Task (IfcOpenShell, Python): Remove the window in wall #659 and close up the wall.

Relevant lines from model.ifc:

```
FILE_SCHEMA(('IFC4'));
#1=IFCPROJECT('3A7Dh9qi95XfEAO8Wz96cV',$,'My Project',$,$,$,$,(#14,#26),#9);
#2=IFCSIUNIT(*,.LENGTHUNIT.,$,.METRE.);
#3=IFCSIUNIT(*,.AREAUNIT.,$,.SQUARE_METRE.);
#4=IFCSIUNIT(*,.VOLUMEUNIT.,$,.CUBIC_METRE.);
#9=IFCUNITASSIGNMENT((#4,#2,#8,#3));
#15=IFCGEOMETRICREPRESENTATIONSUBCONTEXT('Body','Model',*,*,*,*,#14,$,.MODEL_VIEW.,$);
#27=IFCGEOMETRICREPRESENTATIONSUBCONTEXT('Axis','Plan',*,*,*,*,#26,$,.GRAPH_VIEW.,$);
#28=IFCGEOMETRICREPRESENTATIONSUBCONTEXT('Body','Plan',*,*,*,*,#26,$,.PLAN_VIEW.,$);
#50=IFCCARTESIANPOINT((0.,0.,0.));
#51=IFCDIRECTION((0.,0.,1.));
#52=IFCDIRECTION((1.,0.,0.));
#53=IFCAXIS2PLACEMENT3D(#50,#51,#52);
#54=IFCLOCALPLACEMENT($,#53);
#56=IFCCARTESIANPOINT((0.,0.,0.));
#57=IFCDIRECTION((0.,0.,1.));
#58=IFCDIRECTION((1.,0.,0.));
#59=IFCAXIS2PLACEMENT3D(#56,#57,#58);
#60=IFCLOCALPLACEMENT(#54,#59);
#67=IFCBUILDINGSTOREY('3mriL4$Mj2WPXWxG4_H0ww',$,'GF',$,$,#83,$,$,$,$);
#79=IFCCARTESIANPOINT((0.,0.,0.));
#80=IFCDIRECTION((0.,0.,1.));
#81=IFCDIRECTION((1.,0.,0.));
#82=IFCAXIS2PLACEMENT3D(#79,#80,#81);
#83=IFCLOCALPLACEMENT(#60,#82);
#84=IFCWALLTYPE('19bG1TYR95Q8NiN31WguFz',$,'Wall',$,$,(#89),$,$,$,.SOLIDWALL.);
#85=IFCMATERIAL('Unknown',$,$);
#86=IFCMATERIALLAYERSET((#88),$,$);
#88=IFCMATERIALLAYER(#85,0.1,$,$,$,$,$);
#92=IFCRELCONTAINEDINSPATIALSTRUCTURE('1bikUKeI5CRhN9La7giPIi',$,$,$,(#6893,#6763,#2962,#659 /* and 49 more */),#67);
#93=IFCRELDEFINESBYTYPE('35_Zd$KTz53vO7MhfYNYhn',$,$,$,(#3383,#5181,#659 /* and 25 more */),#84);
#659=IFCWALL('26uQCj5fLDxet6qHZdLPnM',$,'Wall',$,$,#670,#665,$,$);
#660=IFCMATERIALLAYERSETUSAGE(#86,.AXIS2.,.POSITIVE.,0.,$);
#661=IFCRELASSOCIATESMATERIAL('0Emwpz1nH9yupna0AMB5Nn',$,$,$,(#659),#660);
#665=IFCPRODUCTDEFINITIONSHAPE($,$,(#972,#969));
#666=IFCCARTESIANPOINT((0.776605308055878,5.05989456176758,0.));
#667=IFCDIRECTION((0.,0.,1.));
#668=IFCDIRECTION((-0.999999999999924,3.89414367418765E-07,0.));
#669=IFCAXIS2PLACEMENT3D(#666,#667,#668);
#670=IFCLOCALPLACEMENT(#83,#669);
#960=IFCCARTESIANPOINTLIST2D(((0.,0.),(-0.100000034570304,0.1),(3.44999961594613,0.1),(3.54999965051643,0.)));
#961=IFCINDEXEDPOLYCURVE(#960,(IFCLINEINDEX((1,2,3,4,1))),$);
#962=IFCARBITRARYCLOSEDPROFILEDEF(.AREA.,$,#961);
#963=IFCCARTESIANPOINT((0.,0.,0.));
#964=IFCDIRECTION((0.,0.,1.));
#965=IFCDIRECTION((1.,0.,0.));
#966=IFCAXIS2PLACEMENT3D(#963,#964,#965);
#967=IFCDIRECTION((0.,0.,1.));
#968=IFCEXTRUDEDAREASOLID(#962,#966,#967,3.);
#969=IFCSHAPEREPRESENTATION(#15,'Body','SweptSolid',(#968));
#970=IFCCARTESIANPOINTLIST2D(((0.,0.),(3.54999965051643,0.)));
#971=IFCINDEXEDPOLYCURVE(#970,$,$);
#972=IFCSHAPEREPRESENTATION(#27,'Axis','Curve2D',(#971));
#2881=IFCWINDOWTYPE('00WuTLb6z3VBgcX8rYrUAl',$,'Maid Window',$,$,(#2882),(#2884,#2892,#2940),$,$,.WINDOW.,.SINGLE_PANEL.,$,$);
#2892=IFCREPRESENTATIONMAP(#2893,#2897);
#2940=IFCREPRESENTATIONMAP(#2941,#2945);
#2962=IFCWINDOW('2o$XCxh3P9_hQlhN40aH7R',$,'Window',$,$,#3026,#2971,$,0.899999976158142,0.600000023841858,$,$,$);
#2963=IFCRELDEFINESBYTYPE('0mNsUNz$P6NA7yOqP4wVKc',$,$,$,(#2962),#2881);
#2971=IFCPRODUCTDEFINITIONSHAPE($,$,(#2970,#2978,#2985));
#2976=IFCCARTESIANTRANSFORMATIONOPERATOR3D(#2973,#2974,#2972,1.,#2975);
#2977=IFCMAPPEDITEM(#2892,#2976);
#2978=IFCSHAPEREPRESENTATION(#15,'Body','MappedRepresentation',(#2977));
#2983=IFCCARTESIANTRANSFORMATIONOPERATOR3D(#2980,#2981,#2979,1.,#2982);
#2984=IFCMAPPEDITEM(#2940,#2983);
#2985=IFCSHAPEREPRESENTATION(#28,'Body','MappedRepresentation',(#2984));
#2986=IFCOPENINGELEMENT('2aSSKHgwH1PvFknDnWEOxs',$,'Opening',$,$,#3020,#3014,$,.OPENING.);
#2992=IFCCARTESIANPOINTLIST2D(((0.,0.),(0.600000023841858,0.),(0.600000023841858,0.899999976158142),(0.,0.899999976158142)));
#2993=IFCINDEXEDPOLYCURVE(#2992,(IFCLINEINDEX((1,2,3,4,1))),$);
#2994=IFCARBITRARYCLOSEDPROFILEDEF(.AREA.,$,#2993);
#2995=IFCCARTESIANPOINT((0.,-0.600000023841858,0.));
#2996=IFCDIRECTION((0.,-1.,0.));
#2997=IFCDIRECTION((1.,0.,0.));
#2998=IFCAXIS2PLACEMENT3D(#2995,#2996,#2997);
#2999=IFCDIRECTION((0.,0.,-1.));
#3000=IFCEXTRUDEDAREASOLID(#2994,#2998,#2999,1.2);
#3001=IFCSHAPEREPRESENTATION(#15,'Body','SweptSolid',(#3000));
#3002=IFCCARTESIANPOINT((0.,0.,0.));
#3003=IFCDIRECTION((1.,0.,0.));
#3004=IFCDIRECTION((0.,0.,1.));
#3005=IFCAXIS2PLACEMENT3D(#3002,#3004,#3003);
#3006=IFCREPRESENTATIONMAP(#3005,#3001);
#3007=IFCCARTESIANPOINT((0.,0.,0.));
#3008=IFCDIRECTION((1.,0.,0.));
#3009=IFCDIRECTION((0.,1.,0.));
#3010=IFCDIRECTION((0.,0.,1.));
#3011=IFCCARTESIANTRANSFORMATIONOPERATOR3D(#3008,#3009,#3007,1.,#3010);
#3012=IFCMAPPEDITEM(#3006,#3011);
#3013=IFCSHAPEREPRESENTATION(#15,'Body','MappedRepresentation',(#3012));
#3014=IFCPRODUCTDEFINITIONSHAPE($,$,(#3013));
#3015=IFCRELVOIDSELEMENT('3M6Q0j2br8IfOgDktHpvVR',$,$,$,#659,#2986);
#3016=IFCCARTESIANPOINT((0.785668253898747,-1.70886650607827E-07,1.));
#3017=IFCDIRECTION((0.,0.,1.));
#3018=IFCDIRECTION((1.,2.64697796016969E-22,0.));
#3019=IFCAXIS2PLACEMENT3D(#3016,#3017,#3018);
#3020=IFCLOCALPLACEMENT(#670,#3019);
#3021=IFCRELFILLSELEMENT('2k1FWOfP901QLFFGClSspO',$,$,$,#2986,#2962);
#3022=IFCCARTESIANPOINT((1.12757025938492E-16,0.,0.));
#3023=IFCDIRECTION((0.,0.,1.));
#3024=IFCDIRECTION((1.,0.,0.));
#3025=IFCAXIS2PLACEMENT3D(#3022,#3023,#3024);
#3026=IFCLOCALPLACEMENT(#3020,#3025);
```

```python
import ifcopenshell
import ifcopenshell.api.feature
import ifcopenshell.api.root
import ifcopenshell.geom
import ifcopenshell.util.shape

model = ifcopenshell.open("model.ifc")
settings = ifcopenshell.geom.settings()


def volume(element):
    """Net volume in cubic metres, openings subtracted."""
    shape = ifcopenshell.geom.create_shape(settings, element)
    return ifcopenshell.util.shape.get_volume(shape.geometry)


window = model.by_guid("2o$XCxh3P9_hQlhN40aH7R")
opening = window.FillsVoids[0].RelatingOpeningElement
wall = opening.VoidsElements[0].RelatingBuildingElement
before = volume(wall)

ifcopenshell.api.root.remove_product(model, product=window)
ifcopenshell.api.feature.remove_feature(model, feature=opening)

after = volume(wall)

print(f"wall volume {before:.3f} -> {after:.3f} m3")

model.write("model_rev.ifc")
```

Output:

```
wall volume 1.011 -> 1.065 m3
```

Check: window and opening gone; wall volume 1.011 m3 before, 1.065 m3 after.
